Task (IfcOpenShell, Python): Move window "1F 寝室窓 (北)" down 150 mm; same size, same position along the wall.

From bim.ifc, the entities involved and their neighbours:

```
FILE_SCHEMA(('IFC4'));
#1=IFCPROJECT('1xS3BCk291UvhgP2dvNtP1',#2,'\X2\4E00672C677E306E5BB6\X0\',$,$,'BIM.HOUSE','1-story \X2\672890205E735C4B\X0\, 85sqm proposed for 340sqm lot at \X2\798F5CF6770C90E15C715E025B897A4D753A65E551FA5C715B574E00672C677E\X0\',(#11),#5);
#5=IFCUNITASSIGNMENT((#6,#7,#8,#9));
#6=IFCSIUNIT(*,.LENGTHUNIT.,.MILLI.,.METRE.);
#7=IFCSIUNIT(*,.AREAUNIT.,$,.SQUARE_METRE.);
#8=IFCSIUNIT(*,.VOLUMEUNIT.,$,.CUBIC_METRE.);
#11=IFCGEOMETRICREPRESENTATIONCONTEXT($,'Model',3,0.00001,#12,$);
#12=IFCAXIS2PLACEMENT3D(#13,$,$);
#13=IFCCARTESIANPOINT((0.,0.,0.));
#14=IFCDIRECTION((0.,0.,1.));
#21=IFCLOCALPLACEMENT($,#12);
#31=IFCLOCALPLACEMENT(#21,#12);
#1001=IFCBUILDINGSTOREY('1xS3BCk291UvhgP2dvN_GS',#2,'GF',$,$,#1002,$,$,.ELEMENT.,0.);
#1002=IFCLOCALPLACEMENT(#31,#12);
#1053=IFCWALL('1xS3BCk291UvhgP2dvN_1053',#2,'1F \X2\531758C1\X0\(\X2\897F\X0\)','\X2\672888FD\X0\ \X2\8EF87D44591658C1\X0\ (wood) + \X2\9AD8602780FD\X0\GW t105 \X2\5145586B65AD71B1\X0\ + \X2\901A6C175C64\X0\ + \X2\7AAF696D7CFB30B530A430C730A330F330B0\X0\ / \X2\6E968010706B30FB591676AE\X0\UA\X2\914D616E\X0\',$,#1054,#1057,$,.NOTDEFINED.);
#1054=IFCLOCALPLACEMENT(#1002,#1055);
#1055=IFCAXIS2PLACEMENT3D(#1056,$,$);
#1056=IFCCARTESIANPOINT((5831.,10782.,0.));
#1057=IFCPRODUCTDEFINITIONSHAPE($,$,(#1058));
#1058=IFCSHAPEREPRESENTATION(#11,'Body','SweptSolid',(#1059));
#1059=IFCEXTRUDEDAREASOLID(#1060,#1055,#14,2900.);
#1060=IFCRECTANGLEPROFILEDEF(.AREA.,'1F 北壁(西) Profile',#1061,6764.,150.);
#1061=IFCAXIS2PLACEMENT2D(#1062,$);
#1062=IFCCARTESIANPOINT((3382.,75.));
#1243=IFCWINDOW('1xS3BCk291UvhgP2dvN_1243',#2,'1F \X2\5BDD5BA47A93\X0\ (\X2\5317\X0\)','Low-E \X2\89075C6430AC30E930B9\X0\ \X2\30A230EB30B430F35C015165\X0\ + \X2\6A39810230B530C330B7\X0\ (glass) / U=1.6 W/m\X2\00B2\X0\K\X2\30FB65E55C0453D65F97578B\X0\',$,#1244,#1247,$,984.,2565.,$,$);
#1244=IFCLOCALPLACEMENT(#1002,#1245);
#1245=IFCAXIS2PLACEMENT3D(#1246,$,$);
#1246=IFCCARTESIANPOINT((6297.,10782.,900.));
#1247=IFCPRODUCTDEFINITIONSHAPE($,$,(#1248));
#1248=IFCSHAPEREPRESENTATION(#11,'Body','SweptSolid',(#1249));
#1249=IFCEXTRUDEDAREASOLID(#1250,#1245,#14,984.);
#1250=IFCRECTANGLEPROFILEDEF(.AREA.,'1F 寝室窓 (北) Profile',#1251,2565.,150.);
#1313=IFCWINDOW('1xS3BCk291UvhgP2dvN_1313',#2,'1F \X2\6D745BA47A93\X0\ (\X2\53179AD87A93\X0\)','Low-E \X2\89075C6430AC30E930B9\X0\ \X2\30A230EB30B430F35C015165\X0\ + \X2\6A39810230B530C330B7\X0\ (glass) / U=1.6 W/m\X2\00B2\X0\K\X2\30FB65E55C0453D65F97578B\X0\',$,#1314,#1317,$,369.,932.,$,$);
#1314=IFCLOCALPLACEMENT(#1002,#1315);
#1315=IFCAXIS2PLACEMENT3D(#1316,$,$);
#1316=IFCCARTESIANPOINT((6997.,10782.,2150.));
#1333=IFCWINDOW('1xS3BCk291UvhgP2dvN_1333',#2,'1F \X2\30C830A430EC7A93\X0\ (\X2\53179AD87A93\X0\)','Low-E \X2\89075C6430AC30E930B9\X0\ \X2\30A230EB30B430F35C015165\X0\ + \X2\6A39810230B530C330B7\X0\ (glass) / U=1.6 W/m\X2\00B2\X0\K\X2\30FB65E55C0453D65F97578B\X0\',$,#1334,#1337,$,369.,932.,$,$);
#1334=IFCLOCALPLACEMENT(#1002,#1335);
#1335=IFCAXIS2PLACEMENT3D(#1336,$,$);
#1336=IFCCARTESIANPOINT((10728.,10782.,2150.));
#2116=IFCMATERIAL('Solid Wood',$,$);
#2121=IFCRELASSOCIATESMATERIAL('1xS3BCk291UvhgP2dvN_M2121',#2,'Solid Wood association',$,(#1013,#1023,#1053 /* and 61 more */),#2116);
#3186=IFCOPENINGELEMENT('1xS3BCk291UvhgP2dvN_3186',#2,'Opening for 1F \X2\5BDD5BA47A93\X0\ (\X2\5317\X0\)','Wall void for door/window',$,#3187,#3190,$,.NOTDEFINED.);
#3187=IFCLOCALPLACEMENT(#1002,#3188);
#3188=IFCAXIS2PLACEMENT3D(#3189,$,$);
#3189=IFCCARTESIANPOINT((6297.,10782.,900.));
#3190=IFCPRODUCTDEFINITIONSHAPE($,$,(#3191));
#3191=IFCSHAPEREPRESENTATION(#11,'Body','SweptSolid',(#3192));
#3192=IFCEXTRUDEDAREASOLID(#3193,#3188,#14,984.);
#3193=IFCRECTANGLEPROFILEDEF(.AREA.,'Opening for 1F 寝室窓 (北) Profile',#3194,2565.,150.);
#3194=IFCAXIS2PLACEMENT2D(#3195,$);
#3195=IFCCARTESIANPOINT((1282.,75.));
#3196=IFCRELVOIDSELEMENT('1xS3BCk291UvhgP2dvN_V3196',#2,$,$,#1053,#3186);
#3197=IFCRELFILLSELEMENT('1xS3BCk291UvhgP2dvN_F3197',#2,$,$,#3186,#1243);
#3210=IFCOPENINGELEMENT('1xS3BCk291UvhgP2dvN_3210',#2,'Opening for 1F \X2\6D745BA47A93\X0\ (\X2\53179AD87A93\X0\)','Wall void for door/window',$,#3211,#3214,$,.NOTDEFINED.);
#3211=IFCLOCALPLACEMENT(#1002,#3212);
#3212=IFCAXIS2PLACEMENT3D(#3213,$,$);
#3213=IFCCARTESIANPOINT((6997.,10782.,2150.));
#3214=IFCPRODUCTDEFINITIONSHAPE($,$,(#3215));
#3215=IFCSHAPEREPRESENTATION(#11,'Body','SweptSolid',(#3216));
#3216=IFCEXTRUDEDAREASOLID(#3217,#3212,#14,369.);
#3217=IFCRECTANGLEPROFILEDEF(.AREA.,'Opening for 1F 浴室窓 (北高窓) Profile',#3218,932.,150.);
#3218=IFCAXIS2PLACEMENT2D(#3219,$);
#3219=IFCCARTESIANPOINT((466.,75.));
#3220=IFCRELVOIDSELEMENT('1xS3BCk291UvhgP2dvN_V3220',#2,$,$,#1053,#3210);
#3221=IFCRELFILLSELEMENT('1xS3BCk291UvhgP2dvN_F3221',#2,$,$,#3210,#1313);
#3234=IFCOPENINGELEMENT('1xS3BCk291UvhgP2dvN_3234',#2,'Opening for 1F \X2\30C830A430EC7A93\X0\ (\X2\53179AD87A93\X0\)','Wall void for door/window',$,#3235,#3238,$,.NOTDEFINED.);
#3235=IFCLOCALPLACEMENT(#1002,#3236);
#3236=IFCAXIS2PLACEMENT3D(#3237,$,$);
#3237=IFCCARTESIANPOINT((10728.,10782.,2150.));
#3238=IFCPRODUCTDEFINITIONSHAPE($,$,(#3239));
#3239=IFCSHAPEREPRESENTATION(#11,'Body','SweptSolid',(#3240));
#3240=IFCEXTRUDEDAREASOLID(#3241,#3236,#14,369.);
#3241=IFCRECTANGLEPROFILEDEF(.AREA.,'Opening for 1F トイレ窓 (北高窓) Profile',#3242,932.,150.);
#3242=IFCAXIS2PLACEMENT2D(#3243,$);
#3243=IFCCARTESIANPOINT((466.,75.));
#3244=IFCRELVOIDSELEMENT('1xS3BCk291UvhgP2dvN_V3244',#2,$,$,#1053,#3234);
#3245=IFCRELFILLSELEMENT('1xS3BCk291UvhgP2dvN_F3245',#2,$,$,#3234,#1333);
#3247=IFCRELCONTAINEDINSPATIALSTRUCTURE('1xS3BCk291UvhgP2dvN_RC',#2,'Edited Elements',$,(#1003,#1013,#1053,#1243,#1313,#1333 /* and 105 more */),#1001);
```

```python
import numpy as np
import ifcopenshell
import ifcopenshell.api.geometry
import ifcopenshell.util.placement
import ifcopenshell.util.unit

model = ifcopenshell.open("bim.ifc")
unit_scale = ifcopenshell.util.unit.calculate_unit_scale(model)

window = model.by_id(1243)
opening = window.FillsVoids[0].RelatingOpeningElement
dz = -0.15 / unit_scale

shift = np.array([0.0, 0.0, dz])
# The window is not placed relative to its opening, so move both.
for product in (opening, window):
    matrix = ifcopenshell.util.placement.get_local_placement(product.ObjectPlacement)
    matrix[:3, 3] += shift
    ifcopenshell.api.geometry.edit_object_placement(model, product=product, matrix=matrix, is_si=False)

print(f"moved by {dz * unit_scale:+.3f} m")

model.write("bim_v2.ifc")
```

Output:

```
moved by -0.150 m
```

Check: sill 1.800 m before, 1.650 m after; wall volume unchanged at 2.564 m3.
